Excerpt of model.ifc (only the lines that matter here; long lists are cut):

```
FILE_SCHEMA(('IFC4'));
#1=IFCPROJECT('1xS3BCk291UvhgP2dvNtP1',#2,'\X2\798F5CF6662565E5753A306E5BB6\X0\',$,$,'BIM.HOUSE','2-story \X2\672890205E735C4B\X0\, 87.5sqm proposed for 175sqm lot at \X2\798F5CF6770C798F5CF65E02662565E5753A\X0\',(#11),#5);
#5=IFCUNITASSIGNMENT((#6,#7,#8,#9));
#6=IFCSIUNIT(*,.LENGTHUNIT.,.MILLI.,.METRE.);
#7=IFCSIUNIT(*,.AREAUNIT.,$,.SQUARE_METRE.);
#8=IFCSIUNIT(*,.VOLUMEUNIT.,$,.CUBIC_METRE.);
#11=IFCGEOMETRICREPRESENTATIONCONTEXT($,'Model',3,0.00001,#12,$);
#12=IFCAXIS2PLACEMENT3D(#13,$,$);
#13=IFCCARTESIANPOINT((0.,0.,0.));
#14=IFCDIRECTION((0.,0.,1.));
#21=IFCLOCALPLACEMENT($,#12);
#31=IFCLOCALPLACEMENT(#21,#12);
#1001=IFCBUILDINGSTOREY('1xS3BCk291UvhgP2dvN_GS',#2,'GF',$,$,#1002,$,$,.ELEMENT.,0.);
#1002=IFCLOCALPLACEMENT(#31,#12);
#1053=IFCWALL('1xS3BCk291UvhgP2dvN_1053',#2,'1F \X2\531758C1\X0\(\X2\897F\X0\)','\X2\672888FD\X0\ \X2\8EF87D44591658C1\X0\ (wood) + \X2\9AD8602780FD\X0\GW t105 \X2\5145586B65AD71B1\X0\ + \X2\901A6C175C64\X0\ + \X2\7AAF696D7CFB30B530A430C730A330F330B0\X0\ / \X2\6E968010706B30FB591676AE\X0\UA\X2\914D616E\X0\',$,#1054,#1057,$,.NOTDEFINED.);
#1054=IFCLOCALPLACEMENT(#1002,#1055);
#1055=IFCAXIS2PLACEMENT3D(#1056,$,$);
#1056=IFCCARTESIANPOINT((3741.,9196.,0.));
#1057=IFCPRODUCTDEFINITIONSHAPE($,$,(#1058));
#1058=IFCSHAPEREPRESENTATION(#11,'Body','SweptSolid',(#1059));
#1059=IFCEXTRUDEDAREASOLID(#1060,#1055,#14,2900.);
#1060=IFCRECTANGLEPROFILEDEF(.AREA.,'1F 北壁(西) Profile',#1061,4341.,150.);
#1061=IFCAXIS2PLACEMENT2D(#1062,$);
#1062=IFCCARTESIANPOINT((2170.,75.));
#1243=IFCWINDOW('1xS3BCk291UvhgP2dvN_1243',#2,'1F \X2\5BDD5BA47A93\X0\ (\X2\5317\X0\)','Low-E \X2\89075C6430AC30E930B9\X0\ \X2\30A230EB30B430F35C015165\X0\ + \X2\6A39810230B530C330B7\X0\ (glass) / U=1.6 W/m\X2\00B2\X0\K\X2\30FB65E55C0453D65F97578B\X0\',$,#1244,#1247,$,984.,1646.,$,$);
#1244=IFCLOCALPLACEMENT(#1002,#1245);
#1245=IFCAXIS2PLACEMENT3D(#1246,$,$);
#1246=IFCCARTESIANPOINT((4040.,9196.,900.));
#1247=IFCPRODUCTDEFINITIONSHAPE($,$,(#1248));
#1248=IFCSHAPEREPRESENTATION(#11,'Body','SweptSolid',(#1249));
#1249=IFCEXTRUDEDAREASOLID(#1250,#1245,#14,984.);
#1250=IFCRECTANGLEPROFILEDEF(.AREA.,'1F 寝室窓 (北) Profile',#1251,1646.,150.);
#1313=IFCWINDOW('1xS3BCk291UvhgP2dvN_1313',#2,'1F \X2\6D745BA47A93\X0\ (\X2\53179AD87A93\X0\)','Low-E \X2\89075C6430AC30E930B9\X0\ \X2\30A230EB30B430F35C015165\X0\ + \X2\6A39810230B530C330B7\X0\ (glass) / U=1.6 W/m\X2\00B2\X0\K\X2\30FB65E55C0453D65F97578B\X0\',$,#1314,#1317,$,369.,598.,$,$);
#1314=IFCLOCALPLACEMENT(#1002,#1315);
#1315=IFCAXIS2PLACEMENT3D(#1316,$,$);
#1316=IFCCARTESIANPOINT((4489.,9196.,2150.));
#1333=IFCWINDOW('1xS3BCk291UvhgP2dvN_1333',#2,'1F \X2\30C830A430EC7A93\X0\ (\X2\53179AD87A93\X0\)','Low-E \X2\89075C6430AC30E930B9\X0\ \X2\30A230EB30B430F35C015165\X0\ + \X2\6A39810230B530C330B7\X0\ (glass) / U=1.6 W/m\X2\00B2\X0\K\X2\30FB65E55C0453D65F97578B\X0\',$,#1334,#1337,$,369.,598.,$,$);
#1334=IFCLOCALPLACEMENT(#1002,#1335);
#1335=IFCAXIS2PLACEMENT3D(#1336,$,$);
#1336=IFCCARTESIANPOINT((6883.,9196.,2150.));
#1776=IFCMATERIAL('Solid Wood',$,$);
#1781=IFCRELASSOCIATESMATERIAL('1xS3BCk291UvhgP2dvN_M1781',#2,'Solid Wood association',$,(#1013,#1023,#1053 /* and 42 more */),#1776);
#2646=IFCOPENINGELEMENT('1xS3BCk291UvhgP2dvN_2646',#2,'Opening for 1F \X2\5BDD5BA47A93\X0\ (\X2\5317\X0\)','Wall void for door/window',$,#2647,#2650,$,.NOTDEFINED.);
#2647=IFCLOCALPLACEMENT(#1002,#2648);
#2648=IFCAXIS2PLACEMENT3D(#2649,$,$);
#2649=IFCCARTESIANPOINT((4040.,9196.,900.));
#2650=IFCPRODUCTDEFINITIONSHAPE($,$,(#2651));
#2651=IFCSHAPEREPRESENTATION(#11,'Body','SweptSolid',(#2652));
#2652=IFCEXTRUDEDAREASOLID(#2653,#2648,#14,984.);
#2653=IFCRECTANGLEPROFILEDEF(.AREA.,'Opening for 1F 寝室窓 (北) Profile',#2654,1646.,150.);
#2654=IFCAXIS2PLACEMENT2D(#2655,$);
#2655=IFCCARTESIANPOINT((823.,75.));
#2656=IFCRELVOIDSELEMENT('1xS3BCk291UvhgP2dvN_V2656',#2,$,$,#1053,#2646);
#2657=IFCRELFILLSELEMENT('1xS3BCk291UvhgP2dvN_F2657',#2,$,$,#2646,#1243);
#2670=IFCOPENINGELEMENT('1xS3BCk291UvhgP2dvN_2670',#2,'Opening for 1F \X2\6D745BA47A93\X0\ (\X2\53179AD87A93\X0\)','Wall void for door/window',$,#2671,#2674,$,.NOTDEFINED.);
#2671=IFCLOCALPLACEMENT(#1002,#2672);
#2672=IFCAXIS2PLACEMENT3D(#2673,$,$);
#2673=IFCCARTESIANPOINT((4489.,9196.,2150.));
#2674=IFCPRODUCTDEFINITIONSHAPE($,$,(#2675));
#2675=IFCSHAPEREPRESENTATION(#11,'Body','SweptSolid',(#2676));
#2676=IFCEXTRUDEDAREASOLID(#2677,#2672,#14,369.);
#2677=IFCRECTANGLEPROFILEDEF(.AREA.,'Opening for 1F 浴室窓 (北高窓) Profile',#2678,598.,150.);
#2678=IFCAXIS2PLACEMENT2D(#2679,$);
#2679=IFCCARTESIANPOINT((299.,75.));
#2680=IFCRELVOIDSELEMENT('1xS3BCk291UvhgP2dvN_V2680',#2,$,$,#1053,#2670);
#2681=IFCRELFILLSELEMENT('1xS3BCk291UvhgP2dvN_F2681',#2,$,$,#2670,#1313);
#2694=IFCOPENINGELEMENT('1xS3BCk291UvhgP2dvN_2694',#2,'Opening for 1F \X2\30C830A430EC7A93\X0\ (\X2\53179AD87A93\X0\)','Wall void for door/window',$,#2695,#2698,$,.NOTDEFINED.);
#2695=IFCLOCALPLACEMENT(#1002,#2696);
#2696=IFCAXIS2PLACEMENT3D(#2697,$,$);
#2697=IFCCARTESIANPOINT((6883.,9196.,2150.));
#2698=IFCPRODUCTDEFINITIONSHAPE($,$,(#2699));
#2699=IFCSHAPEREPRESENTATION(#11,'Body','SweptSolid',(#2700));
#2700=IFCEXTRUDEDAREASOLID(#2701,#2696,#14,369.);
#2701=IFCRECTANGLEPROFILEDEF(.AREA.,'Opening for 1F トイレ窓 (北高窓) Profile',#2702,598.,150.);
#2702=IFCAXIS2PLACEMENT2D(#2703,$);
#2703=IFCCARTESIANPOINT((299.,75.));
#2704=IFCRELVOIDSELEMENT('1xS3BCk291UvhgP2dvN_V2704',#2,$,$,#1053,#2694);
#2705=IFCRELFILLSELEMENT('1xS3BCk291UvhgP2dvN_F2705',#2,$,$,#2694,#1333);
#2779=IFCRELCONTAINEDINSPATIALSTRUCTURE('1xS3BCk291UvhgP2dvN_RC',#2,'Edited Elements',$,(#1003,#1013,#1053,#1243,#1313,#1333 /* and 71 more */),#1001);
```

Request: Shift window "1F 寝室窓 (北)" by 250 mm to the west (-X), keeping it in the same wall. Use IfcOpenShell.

```python
import ifcopenshell
import ifcopenshell.api.geometry
import ifcopenshell.util.placement
import ifcopenshell.util.unit

model = ifcopenshell.open("model.ifc")
unit_scale = ifcopenshell.util.unit.calculate_unit_scale(model)

window = model.by_guid("1xS3BCk291UvhgP2dvN_1243")
opening = window.FillsVoids[0].RelatingOpeningElement
wall = opening.VoidsElements[0].RelatingBuildingElement

wall_matrix = ifcopenshell.util.placement.get_local_placement(wall.ObjectPlacement)
shift = wall_matrix[:3, 0] * -0.25 / unit_scale
before = ifcopenshell.util.placement.get_local_placement(window.ObjectPlacement)[:3, 3].copy()

# The window is not placed relative to its opening, so move both.
for product in (opening, window):
    matrix = ifcopenshell.util.placement.get_local_placement(product.ObjectPlacement)
    matrix[:3, 3] += shift
    ifcopenshell.api.geometry.edit_object_placement(model, product=product, matrix=matrix, is_si=False)

after = ifcopenshell.util.placement.get_local_placement(window.ObjectPlacement)[:3, 3]
print("window moved by", (after - before).round(3) + 0.0)

model.write("model-out.ifc")
```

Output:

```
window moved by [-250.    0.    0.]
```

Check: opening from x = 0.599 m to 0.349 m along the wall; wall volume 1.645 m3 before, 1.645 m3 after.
